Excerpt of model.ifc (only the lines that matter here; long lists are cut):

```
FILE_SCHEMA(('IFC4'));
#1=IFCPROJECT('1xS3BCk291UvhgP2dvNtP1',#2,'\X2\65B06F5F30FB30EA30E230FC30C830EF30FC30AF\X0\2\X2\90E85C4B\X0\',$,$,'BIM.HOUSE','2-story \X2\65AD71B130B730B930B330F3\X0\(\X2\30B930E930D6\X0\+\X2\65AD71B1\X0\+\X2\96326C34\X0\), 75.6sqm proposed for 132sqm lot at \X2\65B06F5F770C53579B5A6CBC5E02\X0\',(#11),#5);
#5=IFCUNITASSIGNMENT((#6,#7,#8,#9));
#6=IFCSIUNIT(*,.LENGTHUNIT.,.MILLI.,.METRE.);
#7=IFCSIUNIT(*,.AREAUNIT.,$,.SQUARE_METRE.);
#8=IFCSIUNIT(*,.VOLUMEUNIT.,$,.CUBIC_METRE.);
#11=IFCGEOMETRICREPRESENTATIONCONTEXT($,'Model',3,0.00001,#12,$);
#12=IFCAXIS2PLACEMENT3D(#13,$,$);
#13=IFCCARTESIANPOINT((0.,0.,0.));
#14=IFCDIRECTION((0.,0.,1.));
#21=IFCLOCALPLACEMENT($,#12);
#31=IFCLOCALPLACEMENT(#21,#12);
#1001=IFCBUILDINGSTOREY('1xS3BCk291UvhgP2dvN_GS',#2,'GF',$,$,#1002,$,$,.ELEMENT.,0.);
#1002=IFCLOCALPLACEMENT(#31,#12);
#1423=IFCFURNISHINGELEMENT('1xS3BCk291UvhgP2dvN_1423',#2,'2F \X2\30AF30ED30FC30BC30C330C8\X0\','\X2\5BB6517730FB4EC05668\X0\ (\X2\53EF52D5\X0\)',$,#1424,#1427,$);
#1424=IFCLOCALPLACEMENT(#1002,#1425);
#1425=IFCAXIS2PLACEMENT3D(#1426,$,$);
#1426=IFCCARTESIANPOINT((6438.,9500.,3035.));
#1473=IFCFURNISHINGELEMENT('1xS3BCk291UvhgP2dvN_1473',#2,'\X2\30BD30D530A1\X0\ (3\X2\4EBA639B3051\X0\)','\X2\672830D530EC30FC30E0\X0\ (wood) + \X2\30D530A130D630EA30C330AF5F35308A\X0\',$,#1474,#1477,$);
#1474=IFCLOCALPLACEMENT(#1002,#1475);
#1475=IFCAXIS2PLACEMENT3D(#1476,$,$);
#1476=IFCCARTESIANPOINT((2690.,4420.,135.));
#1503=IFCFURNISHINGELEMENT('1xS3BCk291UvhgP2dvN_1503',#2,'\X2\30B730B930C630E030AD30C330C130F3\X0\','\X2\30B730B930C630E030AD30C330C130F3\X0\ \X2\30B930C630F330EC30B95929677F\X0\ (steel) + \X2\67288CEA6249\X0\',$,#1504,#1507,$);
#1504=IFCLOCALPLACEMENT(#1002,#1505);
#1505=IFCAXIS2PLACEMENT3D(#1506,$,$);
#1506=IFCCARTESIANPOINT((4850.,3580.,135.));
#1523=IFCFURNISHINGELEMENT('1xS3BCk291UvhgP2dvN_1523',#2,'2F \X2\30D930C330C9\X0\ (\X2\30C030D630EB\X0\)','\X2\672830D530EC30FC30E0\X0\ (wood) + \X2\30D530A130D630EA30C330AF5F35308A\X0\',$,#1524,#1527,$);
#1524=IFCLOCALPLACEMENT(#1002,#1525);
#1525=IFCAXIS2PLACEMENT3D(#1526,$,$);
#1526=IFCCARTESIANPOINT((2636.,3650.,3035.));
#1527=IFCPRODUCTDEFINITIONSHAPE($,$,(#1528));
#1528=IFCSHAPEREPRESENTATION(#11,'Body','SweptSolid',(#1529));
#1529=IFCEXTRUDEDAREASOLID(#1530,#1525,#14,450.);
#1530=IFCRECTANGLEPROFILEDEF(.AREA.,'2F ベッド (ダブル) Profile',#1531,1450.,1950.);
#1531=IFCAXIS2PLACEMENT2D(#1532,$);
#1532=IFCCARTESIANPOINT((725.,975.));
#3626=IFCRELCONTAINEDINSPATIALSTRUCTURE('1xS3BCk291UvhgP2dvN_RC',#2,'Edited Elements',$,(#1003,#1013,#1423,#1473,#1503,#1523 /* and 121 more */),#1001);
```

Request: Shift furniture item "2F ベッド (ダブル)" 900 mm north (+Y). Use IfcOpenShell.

```python
import ifcopenshell
import ifcopenshell.api.geometry
import ifcopenshell.util.placement
import ifcopenshell.util.unit

model = ifcopenshell.open("model.ifc")
unit_scale = ifcopenshell.util.unit.calculate_unit_scale(model)

item = model.by_guid("1xS3BCk291UvhgP2dvN_1523")
matrix = ifcopenshell.util.placement.get_local_placement(item.ObjectPlacement)
matrix[1, 3] += 0.9 / unit_scale
ifcopenshell.api.geometry.edit_object_placement(model, product=item, matrix=matrix, is_si=False)

print(ifcopenshell.util.placement.get_local_placement(item.ObjectPlacement).round(3) + 0.0)

model.write("model_v2.ifc")
```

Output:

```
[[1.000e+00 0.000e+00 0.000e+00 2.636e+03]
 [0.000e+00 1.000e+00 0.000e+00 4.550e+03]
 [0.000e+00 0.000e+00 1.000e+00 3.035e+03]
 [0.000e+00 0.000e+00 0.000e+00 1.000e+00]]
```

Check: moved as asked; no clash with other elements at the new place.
